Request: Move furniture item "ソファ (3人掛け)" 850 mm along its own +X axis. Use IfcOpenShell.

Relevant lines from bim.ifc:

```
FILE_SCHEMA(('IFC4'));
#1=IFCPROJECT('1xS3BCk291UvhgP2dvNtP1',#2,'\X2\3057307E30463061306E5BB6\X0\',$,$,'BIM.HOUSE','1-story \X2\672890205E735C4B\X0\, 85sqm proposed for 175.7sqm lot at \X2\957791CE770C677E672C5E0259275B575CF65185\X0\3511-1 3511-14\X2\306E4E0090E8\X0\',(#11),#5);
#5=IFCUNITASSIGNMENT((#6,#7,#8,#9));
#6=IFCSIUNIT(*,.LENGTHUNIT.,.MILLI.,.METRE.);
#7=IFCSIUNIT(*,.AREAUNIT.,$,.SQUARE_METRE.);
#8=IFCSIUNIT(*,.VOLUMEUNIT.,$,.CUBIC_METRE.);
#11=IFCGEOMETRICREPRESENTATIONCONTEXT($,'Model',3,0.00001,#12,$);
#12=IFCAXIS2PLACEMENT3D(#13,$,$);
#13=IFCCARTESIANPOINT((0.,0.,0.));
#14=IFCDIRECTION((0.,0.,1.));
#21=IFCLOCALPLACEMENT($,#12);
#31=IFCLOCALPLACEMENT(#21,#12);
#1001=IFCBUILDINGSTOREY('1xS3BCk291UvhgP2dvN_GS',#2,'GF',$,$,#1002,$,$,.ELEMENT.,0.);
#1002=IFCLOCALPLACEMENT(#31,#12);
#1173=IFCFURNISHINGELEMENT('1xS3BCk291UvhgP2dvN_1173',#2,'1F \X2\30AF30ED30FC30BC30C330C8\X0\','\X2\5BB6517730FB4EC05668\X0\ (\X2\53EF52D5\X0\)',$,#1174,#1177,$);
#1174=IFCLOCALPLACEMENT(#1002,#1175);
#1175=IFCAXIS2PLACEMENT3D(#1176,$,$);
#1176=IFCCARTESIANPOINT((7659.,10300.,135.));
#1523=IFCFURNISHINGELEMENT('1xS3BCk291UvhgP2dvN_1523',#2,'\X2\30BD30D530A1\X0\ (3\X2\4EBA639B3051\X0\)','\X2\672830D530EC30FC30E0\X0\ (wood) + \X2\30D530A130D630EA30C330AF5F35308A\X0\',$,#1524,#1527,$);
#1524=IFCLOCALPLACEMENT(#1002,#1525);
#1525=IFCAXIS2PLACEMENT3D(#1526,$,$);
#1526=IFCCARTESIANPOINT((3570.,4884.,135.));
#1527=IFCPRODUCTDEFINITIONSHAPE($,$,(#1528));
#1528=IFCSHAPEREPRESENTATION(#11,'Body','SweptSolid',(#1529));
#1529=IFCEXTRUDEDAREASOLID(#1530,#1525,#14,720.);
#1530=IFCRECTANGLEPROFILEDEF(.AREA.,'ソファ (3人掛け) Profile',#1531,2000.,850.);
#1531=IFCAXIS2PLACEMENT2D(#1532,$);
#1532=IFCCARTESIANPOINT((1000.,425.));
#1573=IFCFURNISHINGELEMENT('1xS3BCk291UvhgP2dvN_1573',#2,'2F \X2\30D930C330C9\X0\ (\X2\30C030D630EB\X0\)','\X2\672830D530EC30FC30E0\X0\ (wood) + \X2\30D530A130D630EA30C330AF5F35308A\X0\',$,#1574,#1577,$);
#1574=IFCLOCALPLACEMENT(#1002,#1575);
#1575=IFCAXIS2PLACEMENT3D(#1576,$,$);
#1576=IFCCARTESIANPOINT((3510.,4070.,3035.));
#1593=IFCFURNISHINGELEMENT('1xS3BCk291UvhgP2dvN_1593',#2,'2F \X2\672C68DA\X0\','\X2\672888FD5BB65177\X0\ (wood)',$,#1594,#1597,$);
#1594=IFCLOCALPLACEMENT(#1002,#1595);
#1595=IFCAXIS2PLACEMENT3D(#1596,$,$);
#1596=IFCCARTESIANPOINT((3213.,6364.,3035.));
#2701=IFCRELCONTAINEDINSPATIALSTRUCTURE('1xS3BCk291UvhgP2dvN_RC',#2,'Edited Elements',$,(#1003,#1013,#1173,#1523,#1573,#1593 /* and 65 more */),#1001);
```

```python
import ifcopenshell
import ifcopenshell.api.geometry
import ifcopenshell.util.placement

model = ifcopenshell.open("bim.ifc")

item = model.by_id(1523)
matrix = ifcopenshell.util.placement.get_local_placement(item.ObjectPlacement)
matrix[:3, 3] += matrix[:3, 0] * 850.0
ifcopenshell.api.geometry.edit_object_placement(model, product=item, matrix=matrix, is_si=False)

print(ifcopenshell.util.placement.get_local_placement(item.ObjectPlacement).round(3) + 0.0)

model.write("bim_rev.ifc")
```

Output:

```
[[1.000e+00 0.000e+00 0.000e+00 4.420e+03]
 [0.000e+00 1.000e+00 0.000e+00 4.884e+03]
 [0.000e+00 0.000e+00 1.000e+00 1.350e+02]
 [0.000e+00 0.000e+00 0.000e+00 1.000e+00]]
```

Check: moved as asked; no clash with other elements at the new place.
